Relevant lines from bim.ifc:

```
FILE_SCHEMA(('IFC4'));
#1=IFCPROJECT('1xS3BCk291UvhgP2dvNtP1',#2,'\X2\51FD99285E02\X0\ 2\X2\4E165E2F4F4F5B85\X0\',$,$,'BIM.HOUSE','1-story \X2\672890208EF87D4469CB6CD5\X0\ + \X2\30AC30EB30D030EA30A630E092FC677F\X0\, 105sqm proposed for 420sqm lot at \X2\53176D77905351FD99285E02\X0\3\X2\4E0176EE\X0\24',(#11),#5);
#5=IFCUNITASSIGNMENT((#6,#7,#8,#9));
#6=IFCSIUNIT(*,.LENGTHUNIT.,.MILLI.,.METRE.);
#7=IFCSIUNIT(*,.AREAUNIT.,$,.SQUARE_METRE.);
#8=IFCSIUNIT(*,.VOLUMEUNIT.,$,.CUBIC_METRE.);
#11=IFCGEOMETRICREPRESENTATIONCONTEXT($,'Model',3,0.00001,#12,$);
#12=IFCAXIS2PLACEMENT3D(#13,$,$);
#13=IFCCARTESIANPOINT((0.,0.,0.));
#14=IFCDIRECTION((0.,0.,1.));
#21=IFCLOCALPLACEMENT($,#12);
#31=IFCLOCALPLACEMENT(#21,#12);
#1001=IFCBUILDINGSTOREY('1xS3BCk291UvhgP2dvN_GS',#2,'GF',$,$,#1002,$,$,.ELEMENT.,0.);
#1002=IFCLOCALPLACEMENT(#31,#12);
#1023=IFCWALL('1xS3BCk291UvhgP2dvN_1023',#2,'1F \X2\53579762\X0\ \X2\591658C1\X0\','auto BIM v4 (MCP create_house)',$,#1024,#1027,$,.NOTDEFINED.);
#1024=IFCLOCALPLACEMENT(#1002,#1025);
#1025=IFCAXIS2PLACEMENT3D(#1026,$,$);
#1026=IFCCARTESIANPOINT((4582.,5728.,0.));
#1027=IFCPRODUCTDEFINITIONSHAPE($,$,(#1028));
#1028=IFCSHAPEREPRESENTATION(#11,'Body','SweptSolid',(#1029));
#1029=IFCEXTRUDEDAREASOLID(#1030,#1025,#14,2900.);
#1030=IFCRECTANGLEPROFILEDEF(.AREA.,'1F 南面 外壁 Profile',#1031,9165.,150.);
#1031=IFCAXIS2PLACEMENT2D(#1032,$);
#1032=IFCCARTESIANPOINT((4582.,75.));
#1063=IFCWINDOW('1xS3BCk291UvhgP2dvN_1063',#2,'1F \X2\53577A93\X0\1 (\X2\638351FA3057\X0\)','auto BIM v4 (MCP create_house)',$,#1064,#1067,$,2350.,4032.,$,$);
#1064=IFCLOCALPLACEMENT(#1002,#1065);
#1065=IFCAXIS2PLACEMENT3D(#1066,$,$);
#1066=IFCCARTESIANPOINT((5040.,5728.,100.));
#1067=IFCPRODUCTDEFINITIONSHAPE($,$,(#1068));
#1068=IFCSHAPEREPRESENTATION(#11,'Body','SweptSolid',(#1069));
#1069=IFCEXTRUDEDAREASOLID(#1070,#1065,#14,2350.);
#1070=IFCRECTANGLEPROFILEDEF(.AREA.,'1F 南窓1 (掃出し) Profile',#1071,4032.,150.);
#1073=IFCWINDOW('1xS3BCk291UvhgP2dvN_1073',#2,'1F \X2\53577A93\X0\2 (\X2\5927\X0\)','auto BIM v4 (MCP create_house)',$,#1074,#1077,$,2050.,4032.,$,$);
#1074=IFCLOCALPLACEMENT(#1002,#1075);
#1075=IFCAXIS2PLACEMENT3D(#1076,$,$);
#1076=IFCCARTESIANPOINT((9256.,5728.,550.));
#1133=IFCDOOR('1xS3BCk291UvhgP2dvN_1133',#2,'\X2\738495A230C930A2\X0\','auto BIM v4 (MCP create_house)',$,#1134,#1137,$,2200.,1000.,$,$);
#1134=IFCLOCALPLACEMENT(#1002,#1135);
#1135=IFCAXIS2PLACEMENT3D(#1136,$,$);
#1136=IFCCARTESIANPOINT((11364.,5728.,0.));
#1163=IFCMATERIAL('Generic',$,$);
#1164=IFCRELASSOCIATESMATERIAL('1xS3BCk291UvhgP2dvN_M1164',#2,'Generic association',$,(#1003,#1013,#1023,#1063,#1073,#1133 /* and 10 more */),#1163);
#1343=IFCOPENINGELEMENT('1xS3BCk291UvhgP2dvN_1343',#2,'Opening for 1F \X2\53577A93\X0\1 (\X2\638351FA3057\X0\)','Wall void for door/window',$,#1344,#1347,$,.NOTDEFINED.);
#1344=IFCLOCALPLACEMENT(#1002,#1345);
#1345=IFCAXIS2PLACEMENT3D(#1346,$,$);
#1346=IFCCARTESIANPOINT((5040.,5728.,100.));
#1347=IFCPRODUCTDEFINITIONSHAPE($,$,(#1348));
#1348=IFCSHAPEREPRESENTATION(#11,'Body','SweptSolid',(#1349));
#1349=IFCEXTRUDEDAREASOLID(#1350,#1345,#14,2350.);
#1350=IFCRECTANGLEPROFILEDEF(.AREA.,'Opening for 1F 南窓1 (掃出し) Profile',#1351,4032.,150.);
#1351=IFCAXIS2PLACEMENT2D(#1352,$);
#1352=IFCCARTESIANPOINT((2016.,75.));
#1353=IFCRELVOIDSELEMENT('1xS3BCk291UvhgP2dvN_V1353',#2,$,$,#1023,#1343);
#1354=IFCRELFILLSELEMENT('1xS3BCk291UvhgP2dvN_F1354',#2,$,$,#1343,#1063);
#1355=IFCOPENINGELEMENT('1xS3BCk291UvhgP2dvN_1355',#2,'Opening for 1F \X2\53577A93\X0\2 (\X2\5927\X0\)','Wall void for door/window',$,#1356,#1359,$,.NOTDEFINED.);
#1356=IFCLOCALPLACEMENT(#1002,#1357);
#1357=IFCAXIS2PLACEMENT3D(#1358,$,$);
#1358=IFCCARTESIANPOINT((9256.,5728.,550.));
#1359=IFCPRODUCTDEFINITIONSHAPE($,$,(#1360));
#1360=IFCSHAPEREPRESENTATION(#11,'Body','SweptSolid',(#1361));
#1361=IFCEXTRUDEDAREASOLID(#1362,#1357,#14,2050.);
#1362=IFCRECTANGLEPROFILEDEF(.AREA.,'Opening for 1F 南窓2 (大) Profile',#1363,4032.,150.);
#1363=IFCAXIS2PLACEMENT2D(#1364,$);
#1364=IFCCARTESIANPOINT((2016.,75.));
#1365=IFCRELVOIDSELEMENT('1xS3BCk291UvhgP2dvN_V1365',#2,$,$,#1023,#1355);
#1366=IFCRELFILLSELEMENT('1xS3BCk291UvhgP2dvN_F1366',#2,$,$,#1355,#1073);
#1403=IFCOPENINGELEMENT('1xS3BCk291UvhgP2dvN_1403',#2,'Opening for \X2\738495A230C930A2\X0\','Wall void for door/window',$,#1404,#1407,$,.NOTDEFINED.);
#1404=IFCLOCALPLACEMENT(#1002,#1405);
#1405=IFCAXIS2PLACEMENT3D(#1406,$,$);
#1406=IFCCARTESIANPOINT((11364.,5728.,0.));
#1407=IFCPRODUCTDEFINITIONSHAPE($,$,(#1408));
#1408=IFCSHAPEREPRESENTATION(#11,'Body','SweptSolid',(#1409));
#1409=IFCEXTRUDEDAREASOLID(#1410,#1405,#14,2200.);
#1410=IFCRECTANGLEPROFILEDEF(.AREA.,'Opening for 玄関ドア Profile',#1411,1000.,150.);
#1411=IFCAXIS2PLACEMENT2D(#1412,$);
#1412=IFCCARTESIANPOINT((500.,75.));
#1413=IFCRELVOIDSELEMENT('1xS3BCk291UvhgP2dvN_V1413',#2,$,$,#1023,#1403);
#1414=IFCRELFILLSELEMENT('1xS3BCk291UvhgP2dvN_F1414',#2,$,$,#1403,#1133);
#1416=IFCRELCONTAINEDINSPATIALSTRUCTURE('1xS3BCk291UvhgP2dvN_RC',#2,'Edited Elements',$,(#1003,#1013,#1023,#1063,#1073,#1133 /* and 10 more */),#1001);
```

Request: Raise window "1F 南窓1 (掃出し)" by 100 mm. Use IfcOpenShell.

```python
import numpy as np
import ifcopenshell
import ifcopenshell.api.geometry
import ifcopenshell.util.placement
import ifcopenshell.util.unit

model = ifcopenshell.open("bim.ifc")
unit_scale = ifcopenshell.util.unit.calculate_unit_scale(model)

window = model.by_id(1063)
opening = window.FillsVoids[0].RelatingOpeningElement
dz = 100.0

shift = np.array([0.0, 0.0, dz])
# The window is not placed relative to its opening, so move both.
for product in (opening, window):
    matrix = ifcopenshell.util.placement.get_local_placement(product.ObjectPlacement)
    matrix[:3, 3] += shift
    ifcopenshell.api.geometry.edit_object_placement(model, product=product, matrix=matrix, is_si=False)

print(f"moved by {dz * unit_scale:+.3f} m")

model.write("bim_updated.ifc")
```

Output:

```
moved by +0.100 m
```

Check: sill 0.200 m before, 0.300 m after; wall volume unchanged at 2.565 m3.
